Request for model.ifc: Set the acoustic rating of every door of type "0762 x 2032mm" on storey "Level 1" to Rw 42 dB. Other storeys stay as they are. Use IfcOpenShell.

First a look at what the model holds.

```python
import ifcopenshell
import ifcopenshell.util.element

model = ifcopenshell.open("model.ifc")
print(model.schema)
storey = next(s for s in model.by_type("IfcBuildingStorey") if s.Name == "Level 1")
doors = [e for e in ifcopenshell.util.element.get_decomposition(storey) if e.is_a("IfcDoor")]
seen = {}
for e in doors:
    element_type = ifcopenshell.util.element.get_type(e)
    key = (element_type.Name if element_type != e and element_type else None, ifcopenshell.util.element.get_pset(e, "Pset_DoorCommon", "AcousticRating"))
    seen[key] = seen.get(key, 0) + 1
for (name, value), count in sorted(seen.items(), key=str):
    print(count, "x", name, "|", value)
```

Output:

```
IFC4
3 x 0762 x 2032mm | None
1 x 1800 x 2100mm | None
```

```python
import ifcopenshell
import ifcopenshell.api.pset
import ifcopenshell.util.element

model = ifcopenshell.open("model.ifc")

storey = next(s for s in model.by_type("IfcBuildingStorey") if s.Name == "Level 1")
doors = [e for e in ifcopenshell.util.element.get_decomposition(storey) if e.is_a("IfcDoor")]

count = 0
for e in doors:
    element_type = ifcopenshell.util.element.get_type(e)
    if element_type in (None, e) or element_type.Name != "0762 x 2032mm":
        continue
    # add_pset returns the element's existing set when there is one.
    pset = ifcopenshell.api.pset.add_pset(model, product=e, name="Pset_DoorCommon")
    ifcopenshell.api.pset.edit_pset(model, pset=pset, properties={"AcousticRating": "Rw 42 dB"})
    count += 1

print(count, "doors updated")

model.write("model_v2.ifc")
```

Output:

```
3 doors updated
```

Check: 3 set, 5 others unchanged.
